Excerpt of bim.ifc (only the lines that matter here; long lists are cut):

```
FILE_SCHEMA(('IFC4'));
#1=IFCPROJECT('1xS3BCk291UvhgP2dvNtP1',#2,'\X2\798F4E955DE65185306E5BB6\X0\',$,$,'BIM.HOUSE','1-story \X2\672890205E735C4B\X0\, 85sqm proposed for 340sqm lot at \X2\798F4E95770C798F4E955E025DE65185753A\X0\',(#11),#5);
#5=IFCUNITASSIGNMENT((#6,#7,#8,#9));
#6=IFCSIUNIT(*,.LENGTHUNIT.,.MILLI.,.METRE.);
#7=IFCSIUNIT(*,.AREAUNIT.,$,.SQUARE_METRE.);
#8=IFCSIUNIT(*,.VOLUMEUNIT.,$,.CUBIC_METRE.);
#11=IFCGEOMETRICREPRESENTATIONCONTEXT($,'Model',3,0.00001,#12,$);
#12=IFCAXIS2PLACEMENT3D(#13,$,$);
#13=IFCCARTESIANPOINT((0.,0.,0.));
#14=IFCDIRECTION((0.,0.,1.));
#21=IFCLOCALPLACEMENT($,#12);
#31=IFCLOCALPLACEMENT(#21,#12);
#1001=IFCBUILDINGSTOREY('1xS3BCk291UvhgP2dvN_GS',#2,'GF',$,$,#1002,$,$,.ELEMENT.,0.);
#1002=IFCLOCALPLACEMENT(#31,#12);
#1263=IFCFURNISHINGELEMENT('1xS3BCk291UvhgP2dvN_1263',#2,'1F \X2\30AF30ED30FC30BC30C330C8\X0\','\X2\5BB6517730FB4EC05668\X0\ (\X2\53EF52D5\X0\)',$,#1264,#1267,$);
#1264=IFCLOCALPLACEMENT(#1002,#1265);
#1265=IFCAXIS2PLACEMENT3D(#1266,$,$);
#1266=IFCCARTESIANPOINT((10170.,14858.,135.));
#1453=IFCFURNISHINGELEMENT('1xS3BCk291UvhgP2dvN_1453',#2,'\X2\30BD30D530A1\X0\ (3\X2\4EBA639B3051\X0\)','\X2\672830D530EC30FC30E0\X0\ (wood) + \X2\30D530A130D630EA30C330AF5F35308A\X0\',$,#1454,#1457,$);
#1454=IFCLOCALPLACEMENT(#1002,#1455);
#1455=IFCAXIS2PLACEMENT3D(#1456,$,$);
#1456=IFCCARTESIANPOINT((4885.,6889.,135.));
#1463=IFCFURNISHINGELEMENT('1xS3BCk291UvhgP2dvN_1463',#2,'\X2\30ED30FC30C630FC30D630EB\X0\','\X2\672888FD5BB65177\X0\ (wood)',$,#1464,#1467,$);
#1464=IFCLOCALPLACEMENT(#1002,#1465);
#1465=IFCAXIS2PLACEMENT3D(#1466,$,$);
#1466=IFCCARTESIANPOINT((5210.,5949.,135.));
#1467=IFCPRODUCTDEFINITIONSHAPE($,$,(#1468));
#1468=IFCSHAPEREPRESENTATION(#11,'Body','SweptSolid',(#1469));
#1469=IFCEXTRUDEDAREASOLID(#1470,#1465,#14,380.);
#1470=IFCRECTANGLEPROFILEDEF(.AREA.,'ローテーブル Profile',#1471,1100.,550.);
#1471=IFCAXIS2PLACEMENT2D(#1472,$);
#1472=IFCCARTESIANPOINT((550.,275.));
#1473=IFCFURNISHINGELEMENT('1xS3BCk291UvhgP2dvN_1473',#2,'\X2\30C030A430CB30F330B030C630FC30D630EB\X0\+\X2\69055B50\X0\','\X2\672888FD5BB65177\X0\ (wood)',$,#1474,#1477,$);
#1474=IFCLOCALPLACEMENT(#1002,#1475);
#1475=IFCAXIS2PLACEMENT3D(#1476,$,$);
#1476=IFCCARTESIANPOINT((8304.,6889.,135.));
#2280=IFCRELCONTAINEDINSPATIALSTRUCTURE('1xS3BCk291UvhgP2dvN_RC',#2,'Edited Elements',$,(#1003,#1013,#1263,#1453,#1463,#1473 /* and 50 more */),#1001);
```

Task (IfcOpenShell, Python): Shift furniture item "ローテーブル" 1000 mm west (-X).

```python
import ifcopenshell
import ifcopenshell.api.geometry
import ifcopenshell.util.placement
import ifcopenshell.util.unit

model = ifcopenshell.open("bim.ifc")
unit_scale = ifcopenshell.util.unit.calculate_unit_scale(model)

item = model.by_guid("1xS3BCk291UvhgP2dvN_1463")
matrix = ifcopenshell.util.placement.get_local_placement(item.ObjectPlacement)
matrix[0, 3] -= 1 / unit_scale
ifcopenshell.api.geometry.edit_object_placement(model, product=item, matrix=matrix, is_si=False)

print(ifcopenshell.util.placement.get_local_placement(item.ObjectPlacement).round(3) + 0.0)

model.write("bim_edited.ifc")
```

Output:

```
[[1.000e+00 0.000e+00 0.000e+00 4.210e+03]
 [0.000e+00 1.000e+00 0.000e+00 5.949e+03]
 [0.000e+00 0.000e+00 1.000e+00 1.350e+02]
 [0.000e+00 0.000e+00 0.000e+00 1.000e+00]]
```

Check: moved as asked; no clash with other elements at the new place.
